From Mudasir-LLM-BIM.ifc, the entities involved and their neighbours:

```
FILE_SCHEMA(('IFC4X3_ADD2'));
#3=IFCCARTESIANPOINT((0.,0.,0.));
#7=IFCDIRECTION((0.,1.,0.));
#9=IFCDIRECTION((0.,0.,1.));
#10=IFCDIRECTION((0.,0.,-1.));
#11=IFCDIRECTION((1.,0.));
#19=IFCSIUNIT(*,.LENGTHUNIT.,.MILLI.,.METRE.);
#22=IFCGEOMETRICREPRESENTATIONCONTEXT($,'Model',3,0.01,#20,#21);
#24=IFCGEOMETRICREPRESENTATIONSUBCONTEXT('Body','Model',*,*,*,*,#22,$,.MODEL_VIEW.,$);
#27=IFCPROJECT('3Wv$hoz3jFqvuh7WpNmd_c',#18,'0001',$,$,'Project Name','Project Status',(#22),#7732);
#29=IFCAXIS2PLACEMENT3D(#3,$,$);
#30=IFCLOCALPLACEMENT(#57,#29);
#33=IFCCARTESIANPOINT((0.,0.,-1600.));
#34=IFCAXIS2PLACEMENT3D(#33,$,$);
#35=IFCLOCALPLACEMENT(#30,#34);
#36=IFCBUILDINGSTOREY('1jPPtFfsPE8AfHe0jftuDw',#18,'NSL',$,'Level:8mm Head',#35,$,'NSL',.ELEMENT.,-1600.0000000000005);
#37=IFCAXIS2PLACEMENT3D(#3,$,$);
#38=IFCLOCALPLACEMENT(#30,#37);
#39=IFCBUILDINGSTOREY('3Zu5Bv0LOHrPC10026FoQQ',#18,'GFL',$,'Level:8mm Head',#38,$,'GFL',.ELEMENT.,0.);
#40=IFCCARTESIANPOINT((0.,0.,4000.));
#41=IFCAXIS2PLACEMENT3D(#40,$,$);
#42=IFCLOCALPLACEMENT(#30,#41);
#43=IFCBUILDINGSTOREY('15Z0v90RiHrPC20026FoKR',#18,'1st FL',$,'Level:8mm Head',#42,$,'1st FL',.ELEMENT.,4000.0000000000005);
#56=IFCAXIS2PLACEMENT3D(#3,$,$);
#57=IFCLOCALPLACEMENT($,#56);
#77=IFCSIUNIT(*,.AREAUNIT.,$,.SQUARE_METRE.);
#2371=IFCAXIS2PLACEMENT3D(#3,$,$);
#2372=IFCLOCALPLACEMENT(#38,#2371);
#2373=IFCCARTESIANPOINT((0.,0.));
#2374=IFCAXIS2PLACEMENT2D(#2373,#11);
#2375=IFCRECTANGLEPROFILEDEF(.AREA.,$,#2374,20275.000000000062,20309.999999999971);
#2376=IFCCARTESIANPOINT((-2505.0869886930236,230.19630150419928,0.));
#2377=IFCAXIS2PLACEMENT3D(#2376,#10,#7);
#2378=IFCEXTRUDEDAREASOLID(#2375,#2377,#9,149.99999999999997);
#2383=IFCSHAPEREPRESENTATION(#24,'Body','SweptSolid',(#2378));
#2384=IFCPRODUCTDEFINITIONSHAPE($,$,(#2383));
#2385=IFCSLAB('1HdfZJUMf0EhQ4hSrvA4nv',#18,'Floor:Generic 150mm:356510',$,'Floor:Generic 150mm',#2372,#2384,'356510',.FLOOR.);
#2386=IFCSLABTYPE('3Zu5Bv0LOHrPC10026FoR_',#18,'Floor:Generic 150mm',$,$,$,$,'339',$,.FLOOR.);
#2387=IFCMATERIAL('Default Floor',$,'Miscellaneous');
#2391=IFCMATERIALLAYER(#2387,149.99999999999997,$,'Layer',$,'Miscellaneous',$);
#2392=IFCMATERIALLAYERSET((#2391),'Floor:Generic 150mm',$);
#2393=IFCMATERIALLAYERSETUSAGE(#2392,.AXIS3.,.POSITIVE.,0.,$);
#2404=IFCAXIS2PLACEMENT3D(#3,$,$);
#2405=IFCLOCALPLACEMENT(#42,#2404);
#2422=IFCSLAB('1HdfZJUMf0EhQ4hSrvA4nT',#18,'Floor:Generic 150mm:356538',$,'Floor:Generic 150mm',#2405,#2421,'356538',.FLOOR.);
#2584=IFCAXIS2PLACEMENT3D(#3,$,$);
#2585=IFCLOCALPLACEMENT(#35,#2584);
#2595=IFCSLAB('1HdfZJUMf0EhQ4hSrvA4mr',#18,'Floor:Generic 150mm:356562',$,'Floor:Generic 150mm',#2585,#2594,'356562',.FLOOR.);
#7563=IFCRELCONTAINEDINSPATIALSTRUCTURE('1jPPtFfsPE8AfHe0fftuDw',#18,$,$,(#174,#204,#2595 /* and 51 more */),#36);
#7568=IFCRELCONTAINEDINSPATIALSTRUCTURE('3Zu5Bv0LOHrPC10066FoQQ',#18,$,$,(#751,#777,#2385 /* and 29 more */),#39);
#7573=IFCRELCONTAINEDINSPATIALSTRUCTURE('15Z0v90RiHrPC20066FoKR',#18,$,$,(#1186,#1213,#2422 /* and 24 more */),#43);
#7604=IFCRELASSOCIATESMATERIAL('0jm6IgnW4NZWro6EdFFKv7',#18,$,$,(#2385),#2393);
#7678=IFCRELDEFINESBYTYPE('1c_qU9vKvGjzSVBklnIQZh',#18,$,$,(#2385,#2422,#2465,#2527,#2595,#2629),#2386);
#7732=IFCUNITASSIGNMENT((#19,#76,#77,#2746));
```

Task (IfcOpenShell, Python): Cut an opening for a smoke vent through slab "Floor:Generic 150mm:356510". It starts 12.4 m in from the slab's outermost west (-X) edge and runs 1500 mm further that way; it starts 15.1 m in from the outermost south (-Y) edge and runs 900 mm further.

```python
import numpy as np
import ifcopenshell
import ifcopenshell.api.feature
import ifcopenshell.api.geometry
import ifcopenshell.api.root
import ifcopenshell.geom
import ifcopenshell.util.placement
import ifcopenshell.util.representation
import ifcopenshell.util.shape
import ifcopenshell.util.unit

model = ifcopenshell.open("Mudasir-LLM-BIM.ifc")
unit_scale = ifcopenshell.util.unit.calculate_unit_scale(model)
settings = ifcopenshell.geom.settings()


def volume(element):
    """Net volume in cubic metres, openings subtracted."""
    shape = ifcopenshell.geom.create_shape(settings, element)
    return ifcopenshell.util.shape.get_volume(shape.geometry)


slab = model.by_guid("1HdfZJUMf0EhQ4hSrvA4nv")
before = volume(slab)

# Extent in the slab's own axes, in metres. The edges named are its -X and -Y sides.
slab_shape = ifcopenshell.geom.create_shape(settings, slab)
vertices = ifcopenshell.util.shape.get_vertices(slab_shape.geometry)
x_min, y_min, bottom = vertices.min(axis=0)
top = vertices[:, 2].max()

opening = ifcopenshell.api.root.create_entity(model, ifc_class="IfcOpeningElement", name="Smoke vent opening", predefined_type="OPENING")
context = ifcopenshell.util.representation.get_context(model, "Model", "Body", "MODEL_VIEW")
width, depth = 1.5, 0.9
outline = [(0.0, 0.0), (width, 0.0), (width, depth), (0.0, depth), (0.0, 0.0)]
# Overshoot both faces by 50 mm so the cut is clean.
shape = ifcopenshell.api.geometry.add_slab_representation(
    model, context=context, depth=top - bottom + 0.1, polyline=outline
)
ifcopenshell.api.geometry.assign_representation(model, product=opening, representation=shape)

matrix = ifcopenshell.util.placement.get_local_placement(slab.ObjectPlacement)
matrix[:, 3] = matrix @ np.append(np.array([x_min + 12.4, y_min + 15.1, bottom - 0.05]) / unit_scale, 1.0)
ifcopenshell.api.geometry.edit_object_placement(model, product=opening, matrix=matrix, is_si=False)
ifcopenshell.api.feature.add_feature(model, feature=opening, element=slab)

after = volume(slab)

print(f"slab volume {before:.3f} -> {after:.3f} m3")

model.write("Mudasir-LLM-BIM_rev.ifc")
```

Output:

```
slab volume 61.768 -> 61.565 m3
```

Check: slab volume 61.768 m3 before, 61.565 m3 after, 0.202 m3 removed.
